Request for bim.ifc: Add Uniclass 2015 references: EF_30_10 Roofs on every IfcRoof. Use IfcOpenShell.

First a look at what the model holds.

```python
import ifcopenshell

model = ifcopenshell.open("bim.ifc")
print(model.schema)
print("classifications:", [c.Name for c in model.by_type("IfcClassification")])
for ifc_class in ("IfcDoor", "IfcRoof", "IfcStair", "IfcWall", "IfcWindow"):
    print(ifc_class, len(model.by_type(ifc_class)))
```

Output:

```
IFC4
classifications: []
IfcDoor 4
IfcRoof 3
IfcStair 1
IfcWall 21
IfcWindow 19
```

```python
import ifcopenshell
import ifcopenshell.api.classification

model = ifcopenshell.open("bim.ifc")

system = ifcopenshell.api.classification.add_classification(model, classification="Uniclass 2015")

codes = {
    "IfcRoof": ("EF_30_10", "Roofs"),
}
for ifc_class, (code, name) in codes.items():
    products = model.by_type(ifc_class)
    ifcopenshell.api.classification.add_reference(
        model, products=products, classification=system, identification=code, name=name
    )
    print(code, len(products))

model.write("bim_edited.ifc")
```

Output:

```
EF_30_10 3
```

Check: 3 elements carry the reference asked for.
